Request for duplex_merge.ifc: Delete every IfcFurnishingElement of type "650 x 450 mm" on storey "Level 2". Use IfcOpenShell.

First a look at what the model holds.

```python
import ifcopenshell
import ifcopenshell.util.element

model = ifcopenshell.open("duplex_merge.ifc")
print(model.schema)
storey = next(s for s in model.by_type("IfcBuildingStorey") if s.Name == "Level 2")
furniture = [e for e in ifcopenshell.util.element.get_decomposition(storey) if e.is_a("IfcFurnishingElement")]
seen = {}
for e in furniture:
    element_type = ifcopenshell.util.element.get_type(e)
    name = element_type.Name if element_type not in (None, e) else None
    seen[name] = seen.get(name, 0) + 1
for name, count in sorted(seen.items(), key=str):
    print(count, "x", name)
```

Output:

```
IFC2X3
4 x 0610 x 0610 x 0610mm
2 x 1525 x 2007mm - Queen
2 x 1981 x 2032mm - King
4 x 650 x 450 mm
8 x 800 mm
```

```python
import ifcopenshell
import ifcopenshell.api.root
import ifcopenshell.util.element

model = ifcopenshell.open("duplex_merge.ifc")

storey = next(s for s in model.by_type("IfcBuildingStorey") if s.Name == "Level 2")
furniture = [e for e in ifcopenshell.util.element.get_decomposition(storey) if e.is_a("IfcFurnishingElement")]
targets = [e for e in furniture if (t := ifcopenshell.util.element.get_type(e)) not in (None, e) and t.Name == "650 x 450 mm"]

for e in targets:
    ifcopenshell.api.root.remove_product(model, product=e)
print(len(targets), "removed")

model.write("duplex_merge_updated.ifc")
```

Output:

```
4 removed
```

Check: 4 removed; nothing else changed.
